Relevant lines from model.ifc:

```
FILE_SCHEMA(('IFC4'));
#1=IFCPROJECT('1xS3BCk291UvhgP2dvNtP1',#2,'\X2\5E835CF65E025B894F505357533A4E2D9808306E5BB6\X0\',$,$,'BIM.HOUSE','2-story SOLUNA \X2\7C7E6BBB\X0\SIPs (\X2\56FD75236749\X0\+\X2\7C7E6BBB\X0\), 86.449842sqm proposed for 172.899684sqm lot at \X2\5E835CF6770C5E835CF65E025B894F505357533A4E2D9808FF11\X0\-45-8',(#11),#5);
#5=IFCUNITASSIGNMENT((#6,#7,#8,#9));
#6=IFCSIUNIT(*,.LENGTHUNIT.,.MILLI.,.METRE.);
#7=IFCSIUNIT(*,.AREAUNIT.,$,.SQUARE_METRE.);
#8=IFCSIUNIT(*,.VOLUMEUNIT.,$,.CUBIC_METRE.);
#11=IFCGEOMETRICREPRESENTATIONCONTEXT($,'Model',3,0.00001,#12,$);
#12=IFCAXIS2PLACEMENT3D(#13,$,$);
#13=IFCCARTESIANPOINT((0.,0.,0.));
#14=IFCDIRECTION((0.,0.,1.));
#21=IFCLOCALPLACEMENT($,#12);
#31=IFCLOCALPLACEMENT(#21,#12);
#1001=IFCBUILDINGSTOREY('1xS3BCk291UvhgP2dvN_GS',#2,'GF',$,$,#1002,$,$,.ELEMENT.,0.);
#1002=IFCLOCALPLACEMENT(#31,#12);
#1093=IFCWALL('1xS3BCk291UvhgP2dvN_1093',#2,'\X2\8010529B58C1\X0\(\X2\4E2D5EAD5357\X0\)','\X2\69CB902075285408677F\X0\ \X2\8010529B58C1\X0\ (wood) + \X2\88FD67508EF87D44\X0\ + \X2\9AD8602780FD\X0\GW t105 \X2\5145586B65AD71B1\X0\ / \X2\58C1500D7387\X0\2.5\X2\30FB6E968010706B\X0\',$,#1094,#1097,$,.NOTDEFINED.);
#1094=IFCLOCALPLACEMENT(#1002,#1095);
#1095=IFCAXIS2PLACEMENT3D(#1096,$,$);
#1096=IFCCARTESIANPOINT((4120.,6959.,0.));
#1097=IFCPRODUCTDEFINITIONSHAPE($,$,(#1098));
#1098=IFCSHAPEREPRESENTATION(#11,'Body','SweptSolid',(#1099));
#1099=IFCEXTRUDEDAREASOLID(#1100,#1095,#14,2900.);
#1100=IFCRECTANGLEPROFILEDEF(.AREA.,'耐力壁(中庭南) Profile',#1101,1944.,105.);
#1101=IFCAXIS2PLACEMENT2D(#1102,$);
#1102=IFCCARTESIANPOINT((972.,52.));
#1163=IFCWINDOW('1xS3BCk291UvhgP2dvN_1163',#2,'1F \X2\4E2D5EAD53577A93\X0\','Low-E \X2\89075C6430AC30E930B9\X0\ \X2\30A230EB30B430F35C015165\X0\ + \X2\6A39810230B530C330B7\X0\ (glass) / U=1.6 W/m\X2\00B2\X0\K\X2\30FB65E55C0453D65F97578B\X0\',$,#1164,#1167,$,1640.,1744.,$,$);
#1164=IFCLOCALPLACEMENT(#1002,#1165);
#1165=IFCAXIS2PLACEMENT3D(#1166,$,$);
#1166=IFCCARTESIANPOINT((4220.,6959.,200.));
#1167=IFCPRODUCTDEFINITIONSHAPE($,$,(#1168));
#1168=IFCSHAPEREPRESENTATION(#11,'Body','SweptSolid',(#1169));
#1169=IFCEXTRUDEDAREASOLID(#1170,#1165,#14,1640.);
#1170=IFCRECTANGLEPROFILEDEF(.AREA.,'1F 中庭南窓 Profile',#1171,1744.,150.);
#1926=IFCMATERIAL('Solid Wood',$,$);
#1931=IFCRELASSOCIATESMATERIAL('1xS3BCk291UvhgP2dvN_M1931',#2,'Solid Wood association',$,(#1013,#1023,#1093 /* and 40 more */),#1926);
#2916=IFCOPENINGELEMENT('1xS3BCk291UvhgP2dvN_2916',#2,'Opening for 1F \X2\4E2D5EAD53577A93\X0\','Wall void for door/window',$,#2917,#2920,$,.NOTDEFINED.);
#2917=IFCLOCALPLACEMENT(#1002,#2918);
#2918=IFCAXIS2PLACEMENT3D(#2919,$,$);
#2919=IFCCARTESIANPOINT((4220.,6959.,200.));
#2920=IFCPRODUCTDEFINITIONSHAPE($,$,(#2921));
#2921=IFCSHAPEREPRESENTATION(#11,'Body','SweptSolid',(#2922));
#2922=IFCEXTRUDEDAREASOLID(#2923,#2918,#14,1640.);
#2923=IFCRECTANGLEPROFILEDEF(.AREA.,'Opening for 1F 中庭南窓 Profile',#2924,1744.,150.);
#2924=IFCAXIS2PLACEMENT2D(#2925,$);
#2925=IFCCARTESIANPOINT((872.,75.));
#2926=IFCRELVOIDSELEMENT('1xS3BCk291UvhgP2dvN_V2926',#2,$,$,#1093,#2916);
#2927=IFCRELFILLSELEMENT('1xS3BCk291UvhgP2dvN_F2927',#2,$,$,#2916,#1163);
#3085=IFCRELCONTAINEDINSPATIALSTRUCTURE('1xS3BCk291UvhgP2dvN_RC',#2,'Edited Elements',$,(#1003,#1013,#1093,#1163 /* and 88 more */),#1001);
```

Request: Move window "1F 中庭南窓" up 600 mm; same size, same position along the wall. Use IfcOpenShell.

```python
import numpy as np
import ifcopenshell
import ifcopenshell.api.geometry
import ifcopenshell.util.placement
import ifcopenshell.util.unit

model = ifcopenshell.open("model.ifc")
unit_scale = ifcopenshell.util.unit.calculate_unit_scale(model)

window = model.by_guid("1xS3BCk291UvhgP2dvN_1163")
opening = window.FillsVoids[0].RelatingOpeningElement
dz = 600.0

shift = np.array([0.0, 0.0, dz])
# The window is not placed relative to its opening, so move both.
for product in (opening, window):
    matrix = ifcopenshell.util.placement.get_local_placement(product.ObjectPlacement)
    matrix[:3, 3] += shift
    ifcopenshell.api.geometry.edit_object_placement(model, product=product, matrix=matrix, is_si=False)

print(f"moved by {dz * unit_scale:+.3f} m")

model.write("model_updated.ifc")
```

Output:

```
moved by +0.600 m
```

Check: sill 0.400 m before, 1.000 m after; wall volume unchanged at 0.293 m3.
